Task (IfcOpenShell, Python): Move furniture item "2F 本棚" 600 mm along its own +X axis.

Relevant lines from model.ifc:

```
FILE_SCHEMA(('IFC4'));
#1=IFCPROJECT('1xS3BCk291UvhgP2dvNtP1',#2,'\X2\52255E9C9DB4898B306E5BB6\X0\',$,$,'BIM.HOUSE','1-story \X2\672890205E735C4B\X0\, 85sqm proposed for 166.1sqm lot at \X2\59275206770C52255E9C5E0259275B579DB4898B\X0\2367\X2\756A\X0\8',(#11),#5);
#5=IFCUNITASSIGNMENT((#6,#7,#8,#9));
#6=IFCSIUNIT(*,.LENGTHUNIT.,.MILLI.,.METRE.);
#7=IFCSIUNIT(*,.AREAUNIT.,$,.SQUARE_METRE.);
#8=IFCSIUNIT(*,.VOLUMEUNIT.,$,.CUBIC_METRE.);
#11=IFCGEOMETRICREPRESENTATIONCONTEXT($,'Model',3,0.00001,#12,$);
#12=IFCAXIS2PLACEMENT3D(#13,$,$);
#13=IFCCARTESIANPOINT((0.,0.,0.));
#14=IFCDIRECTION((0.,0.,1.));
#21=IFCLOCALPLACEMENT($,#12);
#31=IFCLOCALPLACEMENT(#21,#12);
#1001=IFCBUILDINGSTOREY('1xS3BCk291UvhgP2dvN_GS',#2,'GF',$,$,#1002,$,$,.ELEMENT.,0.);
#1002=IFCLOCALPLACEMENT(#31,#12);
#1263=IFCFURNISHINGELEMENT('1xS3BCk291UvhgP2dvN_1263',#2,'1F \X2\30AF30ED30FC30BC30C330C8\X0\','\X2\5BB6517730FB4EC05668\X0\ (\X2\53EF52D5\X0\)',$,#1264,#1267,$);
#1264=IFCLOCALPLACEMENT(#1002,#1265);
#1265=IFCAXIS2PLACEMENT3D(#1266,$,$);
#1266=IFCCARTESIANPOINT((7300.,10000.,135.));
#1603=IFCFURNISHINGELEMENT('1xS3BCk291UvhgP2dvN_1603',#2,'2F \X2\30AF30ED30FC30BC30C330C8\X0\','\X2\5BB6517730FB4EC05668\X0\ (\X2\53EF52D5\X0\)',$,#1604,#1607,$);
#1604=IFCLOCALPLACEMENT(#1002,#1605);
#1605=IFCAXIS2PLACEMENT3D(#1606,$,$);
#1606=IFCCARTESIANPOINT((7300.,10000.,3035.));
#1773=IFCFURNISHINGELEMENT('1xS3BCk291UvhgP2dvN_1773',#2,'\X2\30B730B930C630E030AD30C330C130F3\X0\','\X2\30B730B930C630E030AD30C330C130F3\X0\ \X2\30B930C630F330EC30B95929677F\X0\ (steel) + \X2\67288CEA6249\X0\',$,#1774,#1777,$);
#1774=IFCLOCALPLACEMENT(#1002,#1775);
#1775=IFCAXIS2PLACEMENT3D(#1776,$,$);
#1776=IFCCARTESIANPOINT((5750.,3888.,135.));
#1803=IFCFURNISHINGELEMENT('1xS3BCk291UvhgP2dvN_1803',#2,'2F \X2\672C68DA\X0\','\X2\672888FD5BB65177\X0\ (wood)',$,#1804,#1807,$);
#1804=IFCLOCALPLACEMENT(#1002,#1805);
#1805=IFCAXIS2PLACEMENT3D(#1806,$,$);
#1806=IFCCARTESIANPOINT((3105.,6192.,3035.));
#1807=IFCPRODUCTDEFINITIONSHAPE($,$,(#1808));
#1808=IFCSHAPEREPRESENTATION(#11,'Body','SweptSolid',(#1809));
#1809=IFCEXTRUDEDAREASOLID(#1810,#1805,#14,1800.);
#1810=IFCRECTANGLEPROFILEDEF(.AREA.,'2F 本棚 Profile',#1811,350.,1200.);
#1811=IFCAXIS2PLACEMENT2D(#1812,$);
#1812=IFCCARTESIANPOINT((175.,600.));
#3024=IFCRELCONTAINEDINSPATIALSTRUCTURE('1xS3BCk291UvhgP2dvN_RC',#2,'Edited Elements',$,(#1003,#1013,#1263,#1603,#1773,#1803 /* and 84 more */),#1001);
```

```python
import ifcopenshell
import ifcopenshell.api.geometry
import ifcopenshell.util.placement

model = ifcopenshell.open("model.ifc")

item = model.by_id(1803)
matrix = ifcopenshell.util.placement.get_local_placement(item.ObjectPlacement)
matrix[:3, 3] += matrix[:3, 0] * 600.0
ifcopenshell.api.geometry.edit_object_placement(model, product=item, matrix=matrix, is_si=False)

print(ifcopenshell.util.placement.get_local_placement(item.ObjectPlacement).round(3) + 0.0)

model.write("model_rev.ifc")
```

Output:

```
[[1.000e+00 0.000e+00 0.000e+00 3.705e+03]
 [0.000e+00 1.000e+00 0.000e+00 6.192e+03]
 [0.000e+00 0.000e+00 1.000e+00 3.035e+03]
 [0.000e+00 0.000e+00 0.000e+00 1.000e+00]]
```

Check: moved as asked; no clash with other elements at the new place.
